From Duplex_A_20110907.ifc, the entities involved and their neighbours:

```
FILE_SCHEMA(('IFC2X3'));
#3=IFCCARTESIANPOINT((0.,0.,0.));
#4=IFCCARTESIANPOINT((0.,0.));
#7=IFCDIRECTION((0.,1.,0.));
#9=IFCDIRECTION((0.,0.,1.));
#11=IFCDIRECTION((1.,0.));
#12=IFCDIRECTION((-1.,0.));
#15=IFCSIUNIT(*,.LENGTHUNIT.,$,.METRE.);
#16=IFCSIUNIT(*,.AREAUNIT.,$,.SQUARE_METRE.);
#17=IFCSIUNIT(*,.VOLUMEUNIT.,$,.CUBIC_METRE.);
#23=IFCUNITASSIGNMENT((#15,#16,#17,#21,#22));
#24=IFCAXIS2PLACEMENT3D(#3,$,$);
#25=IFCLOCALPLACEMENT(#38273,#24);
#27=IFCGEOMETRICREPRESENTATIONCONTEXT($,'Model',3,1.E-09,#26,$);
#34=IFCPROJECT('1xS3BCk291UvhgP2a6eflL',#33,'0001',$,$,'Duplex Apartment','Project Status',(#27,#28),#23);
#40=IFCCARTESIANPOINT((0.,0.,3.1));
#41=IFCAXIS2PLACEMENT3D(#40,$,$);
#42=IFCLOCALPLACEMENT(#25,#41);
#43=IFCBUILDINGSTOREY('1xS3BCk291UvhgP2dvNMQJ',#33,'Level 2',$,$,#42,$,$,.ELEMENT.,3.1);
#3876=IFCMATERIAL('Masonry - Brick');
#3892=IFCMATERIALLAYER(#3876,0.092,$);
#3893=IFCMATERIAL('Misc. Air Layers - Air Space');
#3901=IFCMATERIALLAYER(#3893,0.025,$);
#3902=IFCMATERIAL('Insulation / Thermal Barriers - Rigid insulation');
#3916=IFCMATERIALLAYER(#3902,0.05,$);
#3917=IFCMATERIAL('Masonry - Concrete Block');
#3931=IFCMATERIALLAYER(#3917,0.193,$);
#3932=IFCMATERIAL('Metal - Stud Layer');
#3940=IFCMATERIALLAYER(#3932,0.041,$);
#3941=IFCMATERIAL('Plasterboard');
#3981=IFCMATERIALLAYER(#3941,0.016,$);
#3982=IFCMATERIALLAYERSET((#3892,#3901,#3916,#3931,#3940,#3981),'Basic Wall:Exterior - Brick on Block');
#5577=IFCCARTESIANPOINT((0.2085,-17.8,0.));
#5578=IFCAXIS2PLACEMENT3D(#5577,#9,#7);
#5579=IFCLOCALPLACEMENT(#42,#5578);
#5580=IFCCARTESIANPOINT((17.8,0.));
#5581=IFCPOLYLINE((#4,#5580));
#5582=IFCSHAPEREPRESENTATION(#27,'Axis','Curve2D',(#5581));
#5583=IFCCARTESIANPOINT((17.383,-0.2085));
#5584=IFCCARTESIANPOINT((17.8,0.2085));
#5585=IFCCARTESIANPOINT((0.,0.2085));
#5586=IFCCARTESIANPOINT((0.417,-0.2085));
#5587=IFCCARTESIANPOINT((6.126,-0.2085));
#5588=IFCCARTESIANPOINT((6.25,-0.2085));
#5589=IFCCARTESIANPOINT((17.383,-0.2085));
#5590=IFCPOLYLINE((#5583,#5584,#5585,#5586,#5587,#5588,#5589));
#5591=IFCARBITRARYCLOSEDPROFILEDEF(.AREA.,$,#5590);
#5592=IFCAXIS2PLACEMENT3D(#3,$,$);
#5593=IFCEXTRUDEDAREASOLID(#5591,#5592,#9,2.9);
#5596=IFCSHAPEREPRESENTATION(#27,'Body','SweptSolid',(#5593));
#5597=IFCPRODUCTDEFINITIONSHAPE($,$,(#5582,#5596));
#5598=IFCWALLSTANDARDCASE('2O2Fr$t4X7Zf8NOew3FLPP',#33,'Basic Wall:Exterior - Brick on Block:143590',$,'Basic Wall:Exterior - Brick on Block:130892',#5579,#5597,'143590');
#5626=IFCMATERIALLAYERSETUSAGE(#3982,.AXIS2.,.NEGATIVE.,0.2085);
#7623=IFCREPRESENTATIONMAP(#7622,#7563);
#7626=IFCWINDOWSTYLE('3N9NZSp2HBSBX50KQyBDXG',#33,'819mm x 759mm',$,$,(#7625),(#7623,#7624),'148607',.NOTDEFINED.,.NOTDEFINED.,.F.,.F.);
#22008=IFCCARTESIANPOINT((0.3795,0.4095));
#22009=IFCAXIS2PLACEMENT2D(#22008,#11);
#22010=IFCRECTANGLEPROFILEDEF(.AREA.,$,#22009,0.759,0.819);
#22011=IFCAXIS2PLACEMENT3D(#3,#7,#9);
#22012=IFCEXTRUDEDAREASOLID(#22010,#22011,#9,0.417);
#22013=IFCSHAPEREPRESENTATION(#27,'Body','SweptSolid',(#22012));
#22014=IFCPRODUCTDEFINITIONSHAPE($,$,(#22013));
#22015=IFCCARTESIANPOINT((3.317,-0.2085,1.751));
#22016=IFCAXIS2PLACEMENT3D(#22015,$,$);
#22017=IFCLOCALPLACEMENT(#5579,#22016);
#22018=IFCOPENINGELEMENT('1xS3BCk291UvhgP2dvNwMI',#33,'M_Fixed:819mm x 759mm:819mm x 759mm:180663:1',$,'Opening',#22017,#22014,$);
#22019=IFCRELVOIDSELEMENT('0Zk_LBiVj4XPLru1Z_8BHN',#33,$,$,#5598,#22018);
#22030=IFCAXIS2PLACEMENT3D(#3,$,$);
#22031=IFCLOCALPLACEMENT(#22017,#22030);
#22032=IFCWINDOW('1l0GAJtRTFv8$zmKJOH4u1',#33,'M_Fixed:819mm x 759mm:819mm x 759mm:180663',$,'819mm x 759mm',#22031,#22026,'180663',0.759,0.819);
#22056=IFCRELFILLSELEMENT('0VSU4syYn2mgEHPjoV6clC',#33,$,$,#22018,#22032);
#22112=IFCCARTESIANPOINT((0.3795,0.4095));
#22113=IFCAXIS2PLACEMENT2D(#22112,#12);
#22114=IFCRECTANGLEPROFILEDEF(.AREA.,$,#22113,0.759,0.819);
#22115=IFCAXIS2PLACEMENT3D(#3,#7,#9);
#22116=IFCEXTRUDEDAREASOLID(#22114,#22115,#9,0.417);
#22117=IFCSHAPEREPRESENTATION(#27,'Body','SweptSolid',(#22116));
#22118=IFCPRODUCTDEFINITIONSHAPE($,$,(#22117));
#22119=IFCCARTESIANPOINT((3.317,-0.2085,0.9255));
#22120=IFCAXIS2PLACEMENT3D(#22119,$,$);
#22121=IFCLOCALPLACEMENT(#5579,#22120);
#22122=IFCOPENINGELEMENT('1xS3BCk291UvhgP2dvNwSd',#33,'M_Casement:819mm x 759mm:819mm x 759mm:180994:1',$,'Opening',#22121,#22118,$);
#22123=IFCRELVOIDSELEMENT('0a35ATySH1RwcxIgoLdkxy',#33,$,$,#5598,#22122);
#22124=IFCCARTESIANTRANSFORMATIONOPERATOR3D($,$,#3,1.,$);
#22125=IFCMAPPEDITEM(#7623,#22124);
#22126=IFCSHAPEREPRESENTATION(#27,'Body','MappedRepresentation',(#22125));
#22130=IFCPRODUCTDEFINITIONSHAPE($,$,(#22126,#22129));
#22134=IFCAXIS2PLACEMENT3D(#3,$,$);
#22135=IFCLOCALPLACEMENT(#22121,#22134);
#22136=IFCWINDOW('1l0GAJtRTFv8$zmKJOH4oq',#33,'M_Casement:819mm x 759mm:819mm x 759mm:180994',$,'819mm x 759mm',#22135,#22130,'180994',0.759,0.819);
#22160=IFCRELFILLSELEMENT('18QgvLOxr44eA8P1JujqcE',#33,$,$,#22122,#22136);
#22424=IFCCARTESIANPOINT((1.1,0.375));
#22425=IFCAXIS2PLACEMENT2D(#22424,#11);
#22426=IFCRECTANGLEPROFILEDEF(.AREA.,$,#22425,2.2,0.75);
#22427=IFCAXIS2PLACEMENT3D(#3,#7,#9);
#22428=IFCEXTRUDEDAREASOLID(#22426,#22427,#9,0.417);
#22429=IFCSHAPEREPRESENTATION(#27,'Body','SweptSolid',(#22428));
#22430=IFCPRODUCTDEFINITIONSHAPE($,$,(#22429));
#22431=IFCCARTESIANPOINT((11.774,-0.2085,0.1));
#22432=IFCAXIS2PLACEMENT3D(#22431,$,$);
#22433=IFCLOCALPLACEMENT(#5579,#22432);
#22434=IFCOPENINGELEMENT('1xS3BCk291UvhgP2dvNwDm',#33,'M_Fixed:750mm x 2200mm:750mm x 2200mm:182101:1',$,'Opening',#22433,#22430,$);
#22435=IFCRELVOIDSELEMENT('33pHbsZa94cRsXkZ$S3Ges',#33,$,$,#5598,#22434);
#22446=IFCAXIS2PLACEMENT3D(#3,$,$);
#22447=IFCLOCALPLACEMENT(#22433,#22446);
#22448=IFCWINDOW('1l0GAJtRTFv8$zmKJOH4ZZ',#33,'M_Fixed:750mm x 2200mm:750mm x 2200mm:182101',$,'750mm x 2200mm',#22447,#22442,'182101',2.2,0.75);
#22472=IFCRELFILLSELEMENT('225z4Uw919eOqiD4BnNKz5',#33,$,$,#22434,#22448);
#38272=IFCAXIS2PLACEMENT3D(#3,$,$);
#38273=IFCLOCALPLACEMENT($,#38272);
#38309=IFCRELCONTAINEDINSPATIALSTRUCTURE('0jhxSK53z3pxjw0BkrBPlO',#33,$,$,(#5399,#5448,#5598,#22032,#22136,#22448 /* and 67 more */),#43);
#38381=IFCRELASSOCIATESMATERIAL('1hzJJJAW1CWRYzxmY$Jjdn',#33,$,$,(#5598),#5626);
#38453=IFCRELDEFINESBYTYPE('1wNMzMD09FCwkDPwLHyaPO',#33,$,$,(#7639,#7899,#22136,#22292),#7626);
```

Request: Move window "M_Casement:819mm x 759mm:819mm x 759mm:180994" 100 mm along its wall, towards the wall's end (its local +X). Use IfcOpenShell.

```python
import ifcopenshell
import ifcopenshell.api.geometry
import ifcopenshell.util.placement

model = ifcopenshell.open("Duplex_A_20110907.ifc")

window = model.by_guid("1l0GAJtRTFv8$zmKJOH4oq")
opening = window.FillsVoids[0].RelatingOpeningElement
wall = opening.VoidsElements[0].RelatingBuildingElement

wall_matrix = ifcopenshell.util.placement.get_local_placement(wall.ObjectPlacement)
shift = wall_matrix[:3, 0] * 0.1
before = ifcopenshell.util.placement.get_local_placement(window.ObjectPlacement)[:3, 3].copy()

# The window is placed relative to its opening, so it follows when the opening moves.
matrix = ifcopenshell.util.placement.get_local_placement(opening.ObjectPlacement)
matrix[:3, 3] += shift
ifcopenshell.api.geometry.edit_object_placement(
    model, product=opening, matrix=matrix, is_si=False, should_transform_children=True
)

after = ifcopenshell.util.placement.get_local_placement(window.ObjectPlacement)[:3, 3]
print("window moved by", (after - before).round(3) + 0.0)

model.write("Duplex_A_20110907_updated.ifc")
```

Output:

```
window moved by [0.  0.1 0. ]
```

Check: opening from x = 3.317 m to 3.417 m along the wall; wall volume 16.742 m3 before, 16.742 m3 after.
